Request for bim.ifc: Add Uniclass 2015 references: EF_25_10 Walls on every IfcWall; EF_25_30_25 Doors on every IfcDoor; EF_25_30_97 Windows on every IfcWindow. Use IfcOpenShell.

First a look at what the model holds.

```python
import ifcopenshell

model = ifcopenshell.open("bim.ifc")
print(model.schema)
print("classifications:", [c.Name for c in model.by_type("IfcClassification")])
for ifc_class in ("IfcDoor", "IfcRoof", "IfcStair", "IfcWall", "IfcWindow"):
    print(ifc_class, len(model.by_type(ifc_class)))
```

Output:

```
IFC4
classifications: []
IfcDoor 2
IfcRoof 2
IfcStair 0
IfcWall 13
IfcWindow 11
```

```python
import ifcopenshell
import ifcopenshell.api.classification

model = ifcopenshell.open("bim.ifc")

system = ifcopenshell.api.classification.add_classification(model, classification="Uniclass 2015")

codes = {
    "IfcWall": ("EF_25_10", "Walls"),
    "IfcDoor": ("EF_25_30_25", "Doors"),
    "IfcWindow": ("EF_25_30_97", "Windows"),
}
for ifc_class, (code, name) in codes.items():
    products = model.by_type(ifc_class)
    ifcopenshell.api.classification.add_reference(
        model, products=products, classification=system, identification=code, name=name
    )
    print(code, len(products))

model.write("bim_updated.ifc")
```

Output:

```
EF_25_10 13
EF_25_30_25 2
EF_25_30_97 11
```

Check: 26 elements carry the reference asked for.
